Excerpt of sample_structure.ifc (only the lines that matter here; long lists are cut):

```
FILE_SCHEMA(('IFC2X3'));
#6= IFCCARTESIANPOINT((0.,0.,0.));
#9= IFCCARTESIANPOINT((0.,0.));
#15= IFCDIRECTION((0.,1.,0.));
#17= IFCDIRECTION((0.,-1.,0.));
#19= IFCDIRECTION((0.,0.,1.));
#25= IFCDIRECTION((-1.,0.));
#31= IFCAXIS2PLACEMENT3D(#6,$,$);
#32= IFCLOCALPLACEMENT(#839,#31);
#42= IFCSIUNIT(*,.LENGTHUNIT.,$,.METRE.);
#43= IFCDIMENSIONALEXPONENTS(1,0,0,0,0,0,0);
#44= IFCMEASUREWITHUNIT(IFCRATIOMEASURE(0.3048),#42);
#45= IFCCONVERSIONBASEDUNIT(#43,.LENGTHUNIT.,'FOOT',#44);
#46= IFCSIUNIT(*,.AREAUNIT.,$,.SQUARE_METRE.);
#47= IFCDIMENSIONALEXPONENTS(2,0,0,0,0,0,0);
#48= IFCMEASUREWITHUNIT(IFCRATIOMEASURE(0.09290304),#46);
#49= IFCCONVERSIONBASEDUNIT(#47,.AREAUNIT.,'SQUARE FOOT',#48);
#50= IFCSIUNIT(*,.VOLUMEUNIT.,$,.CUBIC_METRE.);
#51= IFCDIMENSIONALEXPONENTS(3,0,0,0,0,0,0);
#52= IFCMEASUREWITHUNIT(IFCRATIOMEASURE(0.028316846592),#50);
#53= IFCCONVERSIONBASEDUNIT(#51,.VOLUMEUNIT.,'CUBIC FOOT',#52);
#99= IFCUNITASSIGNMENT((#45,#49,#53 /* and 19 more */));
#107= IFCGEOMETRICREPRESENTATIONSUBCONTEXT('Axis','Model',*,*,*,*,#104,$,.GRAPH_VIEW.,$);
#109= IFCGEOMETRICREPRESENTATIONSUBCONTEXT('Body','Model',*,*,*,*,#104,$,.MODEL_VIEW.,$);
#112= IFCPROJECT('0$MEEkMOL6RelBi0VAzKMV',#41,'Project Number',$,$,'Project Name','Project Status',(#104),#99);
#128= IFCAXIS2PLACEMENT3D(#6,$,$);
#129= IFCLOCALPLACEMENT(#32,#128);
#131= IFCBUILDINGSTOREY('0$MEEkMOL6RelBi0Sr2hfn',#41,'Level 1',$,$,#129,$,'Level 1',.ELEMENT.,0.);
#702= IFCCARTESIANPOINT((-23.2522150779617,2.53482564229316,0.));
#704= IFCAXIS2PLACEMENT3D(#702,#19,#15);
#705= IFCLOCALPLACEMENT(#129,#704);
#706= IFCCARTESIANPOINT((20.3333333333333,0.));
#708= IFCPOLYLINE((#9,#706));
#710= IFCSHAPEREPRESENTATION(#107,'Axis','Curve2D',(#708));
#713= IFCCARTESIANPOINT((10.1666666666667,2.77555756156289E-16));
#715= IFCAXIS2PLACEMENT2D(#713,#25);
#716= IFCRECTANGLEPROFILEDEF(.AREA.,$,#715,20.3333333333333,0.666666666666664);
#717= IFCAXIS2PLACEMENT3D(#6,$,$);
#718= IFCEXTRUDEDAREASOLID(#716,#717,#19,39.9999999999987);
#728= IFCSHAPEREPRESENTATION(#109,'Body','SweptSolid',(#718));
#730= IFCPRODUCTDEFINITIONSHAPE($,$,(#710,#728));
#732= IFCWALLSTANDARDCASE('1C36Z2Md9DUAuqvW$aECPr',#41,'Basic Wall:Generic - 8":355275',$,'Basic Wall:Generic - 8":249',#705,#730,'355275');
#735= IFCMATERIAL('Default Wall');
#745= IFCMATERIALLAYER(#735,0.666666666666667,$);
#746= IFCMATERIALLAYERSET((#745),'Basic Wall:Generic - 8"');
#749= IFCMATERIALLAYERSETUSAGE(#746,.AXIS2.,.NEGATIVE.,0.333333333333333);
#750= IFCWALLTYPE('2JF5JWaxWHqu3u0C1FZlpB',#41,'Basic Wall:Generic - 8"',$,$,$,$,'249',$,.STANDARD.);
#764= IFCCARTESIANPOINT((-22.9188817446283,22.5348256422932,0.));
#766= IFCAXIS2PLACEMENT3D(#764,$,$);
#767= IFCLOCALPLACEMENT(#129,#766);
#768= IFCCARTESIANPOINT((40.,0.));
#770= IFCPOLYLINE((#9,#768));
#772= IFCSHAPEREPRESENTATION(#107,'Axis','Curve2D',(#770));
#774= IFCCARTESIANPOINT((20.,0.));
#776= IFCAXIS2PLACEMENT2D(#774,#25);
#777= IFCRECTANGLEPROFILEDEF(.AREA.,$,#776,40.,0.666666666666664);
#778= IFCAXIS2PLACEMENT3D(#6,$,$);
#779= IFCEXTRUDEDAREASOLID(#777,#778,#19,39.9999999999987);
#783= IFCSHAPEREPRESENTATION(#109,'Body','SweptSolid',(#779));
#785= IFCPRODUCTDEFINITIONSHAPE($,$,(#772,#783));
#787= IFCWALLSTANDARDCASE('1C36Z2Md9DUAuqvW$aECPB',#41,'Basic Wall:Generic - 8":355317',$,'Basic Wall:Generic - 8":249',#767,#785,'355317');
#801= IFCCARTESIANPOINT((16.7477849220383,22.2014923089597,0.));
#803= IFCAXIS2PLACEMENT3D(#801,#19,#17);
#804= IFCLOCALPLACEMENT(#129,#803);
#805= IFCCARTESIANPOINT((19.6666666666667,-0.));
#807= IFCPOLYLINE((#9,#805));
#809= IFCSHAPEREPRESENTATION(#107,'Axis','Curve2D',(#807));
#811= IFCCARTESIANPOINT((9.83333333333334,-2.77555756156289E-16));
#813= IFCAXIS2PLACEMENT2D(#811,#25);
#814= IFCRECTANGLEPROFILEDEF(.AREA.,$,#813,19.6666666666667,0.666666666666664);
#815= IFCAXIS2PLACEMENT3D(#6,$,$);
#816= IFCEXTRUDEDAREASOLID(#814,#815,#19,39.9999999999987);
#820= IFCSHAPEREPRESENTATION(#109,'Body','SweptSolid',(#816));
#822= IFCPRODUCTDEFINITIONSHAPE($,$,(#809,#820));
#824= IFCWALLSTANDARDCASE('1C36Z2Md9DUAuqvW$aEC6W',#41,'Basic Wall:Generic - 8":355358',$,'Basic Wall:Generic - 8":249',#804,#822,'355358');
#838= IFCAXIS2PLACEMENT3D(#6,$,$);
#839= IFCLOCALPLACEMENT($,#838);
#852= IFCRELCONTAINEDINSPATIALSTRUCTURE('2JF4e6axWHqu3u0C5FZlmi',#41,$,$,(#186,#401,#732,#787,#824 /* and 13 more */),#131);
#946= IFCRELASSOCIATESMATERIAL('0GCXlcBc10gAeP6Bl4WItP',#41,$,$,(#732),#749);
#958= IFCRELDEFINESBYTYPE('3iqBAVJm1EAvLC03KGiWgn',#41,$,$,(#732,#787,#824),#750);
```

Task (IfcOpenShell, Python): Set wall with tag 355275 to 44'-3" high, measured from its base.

```python
import ifcopenshell
import ifcopenshell.geom
import ifcopenshell.util.representation
import ifcopenshell.util.shape
import ifcopenshell.util.unit

model = ifcopenshell.open("sample_structure.ifc")
unit_scale = ifcopenshell.util.unit.calculate_unit_scale(model)
settings = ifcopenshell.geom.settings()


def volume(element):
    """Net volume in cubic metres, openings subtracted."""
    shape = ifcopenshell.geom.create_shape(settings, element)
    return ifcopenshell.util.shape.get_volume(shape.geometry)


wall = model.by_guid("1C36Z2Md9DUAuqvW$aECPr")
before = volume(wall)

body = ifcopenshell.util.representation.get_representation(wall, "Model", "Body")
solid = body.Items[0]
old_height = solid.Depth
solid.Depth = 531 * 0.0254 / unit_scale
after = volume(wall)

print(f"height {old_height:g} -> {solid.Depth:g}, volume {before:.3f} -> {after:.3f} m3")

model.write("sample_structure_edited.ifc")
```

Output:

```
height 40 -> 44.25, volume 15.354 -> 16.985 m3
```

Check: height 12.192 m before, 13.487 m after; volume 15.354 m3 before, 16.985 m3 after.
